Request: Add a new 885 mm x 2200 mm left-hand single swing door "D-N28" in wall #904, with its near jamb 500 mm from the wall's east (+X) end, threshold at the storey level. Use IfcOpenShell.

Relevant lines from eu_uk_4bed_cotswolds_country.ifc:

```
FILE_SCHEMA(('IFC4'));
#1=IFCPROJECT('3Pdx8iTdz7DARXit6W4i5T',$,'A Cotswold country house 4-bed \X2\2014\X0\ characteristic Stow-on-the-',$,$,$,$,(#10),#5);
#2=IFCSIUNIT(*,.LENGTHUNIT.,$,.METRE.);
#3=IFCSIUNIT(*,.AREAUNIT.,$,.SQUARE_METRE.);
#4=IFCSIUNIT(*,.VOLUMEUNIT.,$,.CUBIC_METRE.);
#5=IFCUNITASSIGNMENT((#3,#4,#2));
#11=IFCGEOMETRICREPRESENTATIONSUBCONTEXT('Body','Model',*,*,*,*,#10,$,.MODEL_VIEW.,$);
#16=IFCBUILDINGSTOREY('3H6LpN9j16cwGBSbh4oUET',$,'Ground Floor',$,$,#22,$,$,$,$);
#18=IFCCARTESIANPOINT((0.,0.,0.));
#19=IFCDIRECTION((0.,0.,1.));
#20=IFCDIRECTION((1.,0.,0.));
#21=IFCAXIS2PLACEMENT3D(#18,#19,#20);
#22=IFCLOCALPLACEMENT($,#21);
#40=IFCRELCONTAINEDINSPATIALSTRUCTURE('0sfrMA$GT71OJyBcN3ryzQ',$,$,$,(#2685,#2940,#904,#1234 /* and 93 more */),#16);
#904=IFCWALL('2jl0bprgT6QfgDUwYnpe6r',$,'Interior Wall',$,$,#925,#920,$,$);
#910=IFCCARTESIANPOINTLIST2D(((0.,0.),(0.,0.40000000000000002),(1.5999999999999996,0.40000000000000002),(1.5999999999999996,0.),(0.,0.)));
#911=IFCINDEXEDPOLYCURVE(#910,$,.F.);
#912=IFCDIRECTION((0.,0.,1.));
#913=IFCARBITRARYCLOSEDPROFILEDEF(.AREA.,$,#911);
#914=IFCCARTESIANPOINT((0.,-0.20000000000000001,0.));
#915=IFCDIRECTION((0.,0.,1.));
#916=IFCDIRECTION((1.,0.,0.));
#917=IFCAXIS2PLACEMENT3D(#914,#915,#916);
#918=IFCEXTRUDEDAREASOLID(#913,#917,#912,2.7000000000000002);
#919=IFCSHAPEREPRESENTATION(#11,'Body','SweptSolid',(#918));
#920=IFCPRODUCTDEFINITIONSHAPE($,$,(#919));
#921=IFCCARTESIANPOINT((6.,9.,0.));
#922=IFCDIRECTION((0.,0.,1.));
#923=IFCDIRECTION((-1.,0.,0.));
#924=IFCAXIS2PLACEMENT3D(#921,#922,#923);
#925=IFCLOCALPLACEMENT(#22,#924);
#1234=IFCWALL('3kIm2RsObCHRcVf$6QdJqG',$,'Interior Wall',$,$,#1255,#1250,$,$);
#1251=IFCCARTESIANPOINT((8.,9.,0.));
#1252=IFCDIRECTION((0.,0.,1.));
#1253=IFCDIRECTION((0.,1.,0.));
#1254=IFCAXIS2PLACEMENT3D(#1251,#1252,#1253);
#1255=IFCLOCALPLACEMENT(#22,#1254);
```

```python
import numpy as np
import ifcopenshell
import ifcopenshell.api.feature
import ifcopenshell.api.geometry
import ifcopenshell.api.root
import ifcopenshell.api.spatial
import ifcopenshell.geom
import ifcopenshell.util.element
import ifcopenshell.util.placement
import ifcopenshell.util.representation
import ifcopenshell.util.shape
import ifcopenshell.util.unit

model = ifcopenshell.open("eu_uk_4bed_cotswolds_country.ifc")
unit_scale = ifcopenshell.util.unit.calculate_unit_scale(model)
settings = ifcopenshell.geom.settings()


def volume(element):
    """Net volume in cubic metres, openings subtracted."""
    shape = ifcopenshell.geom.create_shape(settings, element)
    return ifcopenshell.util.shape.get_volume(shape.geometry)


wall = model.by_guid("2jl0bprgT6QfgDUwYnpe6r")
storey = ifcopenshell.util.element.get_container(wall, ifc_class="IfcBuildingStorey")
context = ifcopenshell.util.representation.get_context(model, "Model", "Body", "MODEL_VIEW")
before = volume(wall)

width, height, from_end, sill = 0.885, 2.2, 0.5, 0.0  # metres

# The wall runs along its own X axis, and the end named is its -X end.
wall_shape = ifcopenshell.geom.create_shape(settings, wall)
x, y, z = ifcopenshell.util.shape.get_vertices(wall_shape.geometry).T
start = x.min() + from_end
face, thickness = float(y.min()), float(y.max() - y.min())
wall_matrix = ifcopenshell.util.placement.get_local_placement(wall.ObjectPlacement)
level = ifcopenshell.util.placement.get_local_placement(storey.ObjectPlacement)[2, 3]


def in_wall(x, y):
    """Placement at x, y metres in the wall's axes, at sill height."""
    matrix = wall_matrix.copy()
    matrix[:, 3] = wall_matrix @ np.array([x / unit_scale, y / unit_scale, 0.0, 1.0])
    matrix[2, 3] = level + sill / unit_scale
    return matrix


# Opening: a box that overshoots both wall faces by 50 mm.
opening = ifcopenshell.api.root.create_entity(model, ifc_class="IfcOpeningElement", predefined_type="OPENING")
box = ifcopenshell.api.geometry.add_wall_representation(
    model, context=context, length=width, height=height, thickness=thickness + 0.1
)
ifcopenshell.api.geometry.assign_representation(model, product=opening, representation=box)
ifcopenshell.api.geometry.edit_object_placement(model, product=opening, matrix=in_wall(start, face - 0.05), is_si=False)
ifcopenshell.api.feature.add_feature(model, feature=opening, element=wall)

door = ifcopenshell.api.root.create_entity(model, ifc_class="IfcDoor", name="D-N28", predefined_type="DOOR")
door.OverallWidth, door.OverallHeight = width / unit_scale, height / unit_scale
door.OperationType = "SINGLE_SWING_LEFT"
body = ifcopenshell.api.geometry.add_door_representation(
    model,
    context=context,
    overall_width=door.OverallWidth,
    overall_height=door.OverallHeight,
    operation_type="SINGLE_SWING_LEFT",
    lining_properties={"LiningDepth": thickness / unit_scale, "ThresholdDepth": thickness / unit_scale},
)
ifcopenshell.api.geometry.assign_representation(model, product=door, representation=body)
ifcopenshell.api.spatial.assign_container(model, products=[door], relating_structure=storey)
ifcopenshell.api.feature.add_filling(model, opening=opening, element=door)

# The lining spans the wall, so the door starts at the wall face.
ifcopenshell.api.geometry.edit_object_placement(model, product=door, matrix=in_wall(start, face), is_si=False)

after = volume(wall)

print(f"wall volume {before:.3f} -> {after:.3f} m3")

model.write("eu_uk_4bed_cotswolds_country_edited.ifc")
```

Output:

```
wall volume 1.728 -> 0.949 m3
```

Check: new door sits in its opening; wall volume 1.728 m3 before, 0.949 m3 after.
